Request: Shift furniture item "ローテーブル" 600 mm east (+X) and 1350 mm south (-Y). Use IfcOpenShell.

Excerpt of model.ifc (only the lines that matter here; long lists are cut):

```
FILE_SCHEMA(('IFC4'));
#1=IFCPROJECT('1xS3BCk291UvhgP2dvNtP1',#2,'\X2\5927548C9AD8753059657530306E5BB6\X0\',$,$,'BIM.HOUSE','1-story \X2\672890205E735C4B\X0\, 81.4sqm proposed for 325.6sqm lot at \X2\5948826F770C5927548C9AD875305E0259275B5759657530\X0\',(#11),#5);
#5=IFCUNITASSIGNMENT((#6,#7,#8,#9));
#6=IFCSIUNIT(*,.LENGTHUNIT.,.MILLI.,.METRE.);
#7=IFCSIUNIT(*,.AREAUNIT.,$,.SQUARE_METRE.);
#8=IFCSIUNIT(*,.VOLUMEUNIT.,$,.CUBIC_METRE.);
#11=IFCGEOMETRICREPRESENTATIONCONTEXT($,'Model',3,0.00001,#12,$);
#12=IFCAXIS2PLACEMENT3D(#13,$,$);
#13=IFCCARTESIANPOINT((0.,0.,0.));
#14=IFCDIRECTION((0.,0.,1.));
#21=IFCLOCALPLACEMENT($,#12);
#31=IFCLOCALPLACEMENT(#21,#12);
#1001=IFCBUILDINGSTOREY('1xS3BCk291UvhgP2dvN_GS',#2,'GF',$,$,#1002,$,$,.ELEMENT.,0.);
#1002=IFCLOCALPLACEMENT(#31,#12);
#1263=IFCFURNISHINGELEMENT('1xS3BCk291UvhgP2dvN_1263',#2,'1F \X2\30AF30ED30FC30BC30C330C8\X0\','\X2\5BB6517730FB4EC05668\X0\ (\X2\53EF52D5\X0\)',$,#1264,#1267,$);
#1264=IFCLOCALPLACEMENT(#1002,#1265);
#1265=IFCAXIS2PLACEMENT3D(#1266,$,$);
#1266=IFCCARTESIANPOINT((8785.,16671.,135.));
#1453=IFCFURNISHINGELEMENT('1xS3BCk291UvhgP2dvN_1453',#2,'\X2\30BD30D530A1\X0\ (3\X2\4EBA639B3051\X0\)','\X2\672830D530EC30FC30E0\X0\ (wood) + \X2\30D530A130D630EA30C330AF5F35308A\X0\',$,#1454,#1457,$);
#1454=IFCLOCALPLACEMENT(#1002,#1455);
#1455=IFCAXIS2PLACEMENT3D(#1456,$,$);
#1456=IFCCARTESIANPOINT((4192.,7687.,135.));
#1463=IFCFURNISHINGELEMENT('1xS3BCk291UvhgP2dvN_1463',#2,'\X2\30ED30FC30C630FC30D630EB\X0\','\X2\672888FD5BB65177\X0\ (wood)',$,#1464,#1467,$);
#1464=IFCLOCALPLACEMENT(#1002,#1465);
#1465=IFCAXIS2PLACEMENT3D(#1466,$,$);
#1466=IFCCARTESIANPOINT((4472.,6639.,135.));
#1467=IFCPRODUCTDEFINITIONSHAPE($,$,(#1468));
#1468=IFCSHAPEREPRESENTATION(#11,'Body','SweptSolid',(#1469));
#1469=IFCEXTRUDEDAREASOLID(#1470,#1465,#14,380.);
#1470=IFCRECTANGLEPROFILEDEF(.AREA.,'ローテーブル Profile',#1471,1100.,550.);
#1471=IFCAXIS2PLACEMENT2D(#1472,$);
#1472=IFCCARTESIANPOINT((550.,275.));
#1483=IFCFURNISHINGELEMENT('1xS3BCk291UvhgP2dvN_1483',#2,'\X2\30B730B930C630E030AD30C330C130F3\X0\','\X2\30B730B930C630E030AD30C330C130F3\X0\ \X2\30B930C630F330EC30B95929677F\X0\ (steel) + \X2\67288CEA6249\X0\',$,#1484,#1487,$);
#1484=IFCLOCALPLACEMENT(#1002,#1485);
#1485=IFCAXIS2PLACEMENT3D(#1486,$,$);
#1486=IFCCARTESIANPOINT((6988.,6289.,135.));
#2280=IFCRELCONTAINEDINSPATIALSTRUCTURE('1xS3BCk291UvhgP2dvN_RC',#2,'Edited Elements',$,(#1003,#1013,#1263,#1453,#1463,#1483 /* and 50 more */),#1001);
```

```python
import ifcopenshell
import ifcopenshell.api.geometry
import ifcopenshell.util.placement

model = ifcopenshell.open("model.ifc")

item = model.by_guid("1xS3BCk291UvhgP2dvN_1463")
matrix = ifcopenshell.util.placement.get_local_placement(item.ObjectPlacement)
matrix[0, 3] += 600.0
matrix[1, 3] -= 1350.0
ifcopenshell.api.geometry.edit_object_placement(model, product=item, matrix=matrix, is_si=False)

print(ifcopenshell.util.placement.get_local_placement(item.ObjectPlacement).round(3) + 0.0)

model.write("model_rev.ifc")
```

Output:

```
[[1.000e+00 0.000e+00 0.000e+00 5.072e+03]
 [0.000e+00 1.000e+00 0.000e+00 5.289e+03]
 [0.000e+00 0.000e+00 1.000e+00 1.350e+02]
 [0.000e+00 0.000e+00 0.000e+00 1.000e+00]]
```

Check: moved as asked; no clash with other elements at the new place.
